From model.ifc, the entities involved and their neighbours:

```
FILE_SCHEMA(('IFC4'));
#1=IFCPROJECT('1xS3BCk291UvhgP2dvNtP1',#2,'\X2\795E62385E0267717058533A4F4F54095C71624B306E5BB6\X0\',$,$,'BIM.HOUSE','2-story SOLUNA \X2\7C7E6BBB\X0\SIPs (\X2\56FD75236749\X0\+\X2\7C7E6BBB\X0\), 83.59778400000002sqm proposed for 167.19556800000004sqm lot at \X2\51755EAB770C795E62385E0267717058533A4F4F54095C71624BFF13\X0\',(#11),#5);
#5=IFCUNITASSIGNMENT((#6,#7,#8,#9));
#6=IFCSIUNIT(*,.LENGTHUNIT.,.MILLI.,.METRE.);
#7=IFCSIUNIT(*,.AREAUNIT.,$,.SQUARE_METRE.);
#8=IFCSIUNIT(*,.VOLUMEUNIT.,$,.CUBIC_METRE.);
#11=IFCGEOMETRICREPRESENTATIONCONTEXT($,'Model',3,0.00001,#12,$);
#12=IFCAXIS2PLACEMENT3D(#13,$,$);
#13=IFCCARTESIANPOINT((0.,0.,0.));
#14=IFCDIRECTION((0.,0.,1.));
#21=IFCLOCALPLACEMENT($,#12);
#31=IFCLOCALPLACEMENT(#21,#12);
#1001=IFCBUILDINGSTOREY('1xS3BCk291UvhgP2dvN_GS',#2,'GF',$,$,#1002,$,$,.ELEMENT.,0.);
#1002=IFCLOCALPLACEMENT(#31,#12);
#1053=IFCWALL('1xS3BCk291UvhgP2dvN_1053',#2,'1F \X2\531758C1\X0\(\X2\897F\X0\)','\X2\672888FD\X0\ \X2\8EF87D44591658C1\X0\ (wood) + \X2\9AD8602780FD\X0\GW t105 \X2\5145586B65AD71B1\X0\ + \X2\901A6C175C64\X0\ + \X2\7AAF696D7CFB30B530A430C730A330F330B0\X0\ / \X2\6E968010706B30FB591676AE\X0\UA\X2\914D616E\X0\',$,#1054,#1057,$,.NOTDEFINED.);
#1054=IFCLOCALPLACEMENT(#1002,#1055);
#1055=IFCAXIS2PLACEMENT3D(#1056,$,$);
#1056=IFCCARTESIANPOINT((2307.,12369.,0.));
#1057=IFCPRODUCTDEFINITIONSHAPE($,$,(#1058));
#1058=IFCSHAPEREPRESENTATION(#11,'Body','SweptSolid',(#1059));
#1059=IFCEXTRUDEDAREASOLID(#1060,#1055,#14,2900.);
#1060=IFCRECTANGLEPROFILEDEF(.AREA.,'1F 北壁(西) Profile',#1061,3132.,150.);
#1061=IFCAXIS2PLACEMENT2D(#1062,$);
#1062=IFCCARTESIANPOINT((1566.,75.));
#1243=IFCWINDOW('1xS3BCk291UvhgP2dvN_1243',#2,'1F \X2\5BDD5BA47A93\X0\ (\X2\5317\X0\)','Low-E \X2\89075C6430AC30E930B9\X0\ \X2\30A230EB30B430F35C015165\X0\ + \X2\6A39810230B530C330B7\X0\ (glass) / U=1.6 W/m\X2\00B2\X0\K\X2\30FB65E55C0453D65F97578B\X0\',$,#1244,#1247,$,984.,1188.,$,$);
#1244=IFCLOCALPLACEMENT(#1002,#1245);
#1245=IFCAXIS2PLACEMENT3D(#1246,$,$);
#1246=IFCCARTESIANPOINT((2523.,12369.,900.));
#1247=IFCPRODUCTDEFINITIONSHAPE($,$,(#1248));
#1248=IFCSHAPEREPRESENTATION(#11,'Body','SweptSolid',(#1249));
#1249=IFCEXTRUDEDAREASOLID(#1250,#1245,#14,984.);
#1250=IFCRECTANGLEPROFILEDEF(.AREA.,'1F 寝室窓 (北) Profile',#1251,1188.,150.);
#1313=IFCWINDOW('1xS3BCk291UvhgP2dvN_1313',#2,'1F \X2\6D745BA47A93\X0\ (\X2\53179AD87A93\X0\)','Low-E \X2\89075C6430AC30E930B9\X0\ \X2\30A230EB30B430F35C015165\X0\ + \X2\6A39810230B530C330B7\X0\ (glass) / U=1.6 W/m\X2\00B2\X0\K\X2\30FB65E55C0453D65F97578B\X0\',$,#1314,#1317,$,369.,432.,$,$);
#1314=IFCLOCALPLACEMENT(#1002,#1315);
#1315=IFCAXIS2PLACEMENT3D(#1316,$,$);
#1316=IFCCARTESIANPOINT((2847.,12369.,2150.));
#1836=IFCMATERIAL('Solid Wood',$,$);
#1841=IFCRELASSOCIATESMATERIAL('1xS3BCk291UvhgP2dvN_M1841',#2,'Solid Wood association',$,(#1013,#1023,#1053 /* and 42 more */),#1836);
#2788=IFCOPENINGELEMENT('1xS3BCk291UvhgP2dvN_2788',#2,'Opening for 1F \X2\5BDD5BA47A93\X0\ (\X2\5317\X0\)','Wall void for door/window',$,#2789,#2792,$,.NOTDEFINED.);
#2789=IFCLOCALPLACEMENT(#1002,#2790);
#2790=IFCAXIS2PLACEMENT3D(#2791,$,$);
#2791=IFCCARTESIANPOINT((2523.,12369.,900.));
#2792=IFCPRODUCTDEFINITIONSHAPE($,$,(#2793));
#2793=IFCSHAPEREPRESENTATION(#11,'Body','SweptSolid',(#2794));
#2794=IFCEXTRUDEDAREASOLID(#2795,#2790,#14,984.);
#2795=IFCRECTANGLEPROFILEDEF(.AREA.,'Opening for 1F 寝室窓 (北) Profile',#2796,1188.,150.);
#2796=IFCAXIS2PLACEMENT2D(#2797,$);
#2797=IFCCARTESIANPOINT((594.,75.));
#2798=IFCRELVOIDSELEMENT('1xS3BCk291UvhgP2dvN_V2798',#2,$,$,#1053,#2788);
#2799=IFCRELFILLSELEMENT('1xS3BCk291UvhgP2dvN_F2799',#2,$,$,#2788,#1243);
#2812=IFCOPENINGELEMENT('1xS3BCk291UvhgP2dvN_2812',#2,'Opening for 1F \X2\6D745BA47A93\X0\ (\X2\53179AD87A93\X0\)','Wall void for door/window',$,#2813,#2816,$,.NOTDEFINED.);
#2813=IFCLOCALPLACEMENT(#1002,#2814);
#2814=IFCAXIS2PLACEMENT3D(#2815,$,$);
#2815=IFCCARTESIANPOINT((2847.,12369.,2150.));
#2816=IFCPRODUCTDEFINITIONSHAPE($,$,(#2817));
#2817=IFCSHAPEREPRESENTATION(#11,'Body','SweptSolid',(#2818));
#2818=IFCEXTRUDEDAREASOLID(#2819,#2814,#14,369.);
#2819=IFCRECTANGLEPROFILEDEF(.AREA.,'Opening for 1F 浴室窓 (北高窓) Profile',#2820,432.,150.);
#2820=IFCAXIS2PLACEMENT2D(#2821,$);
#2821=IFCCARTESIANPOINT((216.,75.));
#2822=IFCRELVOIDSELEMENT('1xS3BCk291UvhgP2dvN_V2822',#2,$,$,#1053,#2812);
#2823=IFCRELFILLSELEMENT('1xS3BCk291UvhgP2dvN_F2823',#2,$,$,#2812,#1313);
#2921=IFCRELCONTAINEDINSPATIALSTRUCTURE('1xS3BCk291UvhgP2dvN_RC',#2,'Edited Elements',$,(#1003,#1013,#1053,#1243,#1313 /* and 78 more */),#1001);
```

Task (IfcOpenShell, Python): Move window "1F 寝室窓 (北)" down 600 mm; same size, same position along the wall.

```python
import numpy as np
import ifcopenshell
import ifcopenshell.api.geometry
import ifcopenshell.util.placement
import ifcopenshell.util.unit

model = ifcopenshell.open("model.ifc")
unit_scale = ifcopenshell.util.unit.calculate_unit_scale(model)

window = model.by_guid("1xS3BCk291UvhgP2dvN_1243")
opening = window.FillsVoids[0].RelatingOpeningElement
dz = -0.6 / unit_scale

shift = np.array([0.0, 0.0, dz])
# The window is not placed relative to its opening, so move both.
for product in (opening, window):
    matrix = ifcopenshell.util.placement.get_local_placement(product.ObjectPlacement)
    matrix[:3, 3] += shift
    ifcopenshell.api.geometry.edit_object_placement(model, product=product, matrix=matrix, is_si=False)

print(f"moved by {dz * unit_scale:+.3f} m")

model.write("model_updated.ifc")
```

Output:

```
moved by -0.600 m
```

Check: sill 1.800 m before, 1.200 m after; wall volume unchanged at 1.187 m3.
